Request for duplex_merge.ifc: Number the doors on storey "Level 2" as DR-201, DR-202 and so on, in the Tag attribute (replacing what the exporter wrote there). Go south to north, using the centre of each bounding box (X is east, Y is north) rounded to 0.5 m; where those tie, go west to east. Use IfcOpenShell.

First a look at what the model holds.

```python
import ifcopenshell
import ifcopenshell.util.element
import ifcopenshell.util.placement

model = ifcopenshell.open("duplex_merge.ifc")
print(model.schema)
storey = next(s for s in model.by_type("IfcBuildingStorey") if s.Name == "Level 2")
doors = [e for e in ifcopenshell.util.element.get_decomposition(storey) if e.is_a("IfcDoor")]
for e in sorted(doors, key=lambda e: e.id()):
    origin = ifcopenshell.util.placement.get_local_placement(e.ObjectPlacement)[:3, 3]
    print(e.id(), e.Tag, e.Name, origin.round(2) + 0.0, sep=" | ")
```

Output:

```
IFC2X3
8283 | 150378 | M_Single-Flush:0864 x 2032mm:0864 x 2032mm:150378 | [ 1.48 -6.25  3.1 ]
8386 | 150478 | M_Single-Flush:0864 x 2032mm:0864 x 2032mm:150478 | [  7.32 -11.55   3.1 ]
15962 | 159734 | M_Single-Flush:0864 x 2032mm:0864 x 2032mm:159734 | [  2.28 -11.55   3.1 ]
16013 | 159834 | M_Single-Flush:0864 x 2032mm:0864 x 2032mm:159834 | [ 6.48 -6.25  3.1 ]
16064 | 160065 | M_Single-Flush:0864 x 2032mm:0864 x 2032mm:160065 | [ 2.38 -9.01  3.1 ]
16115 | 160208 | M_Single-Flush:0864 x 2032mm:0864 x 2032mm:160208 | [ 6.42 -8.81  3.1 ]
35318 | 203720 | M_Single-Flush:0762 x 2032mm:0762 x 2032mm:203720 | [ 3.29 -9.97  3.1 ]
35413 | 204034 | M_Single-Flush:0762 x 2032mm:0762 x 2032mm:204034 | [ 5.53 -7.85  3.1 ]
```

```python
import ifcopenshell
import ifcopenshell.geom
import ifcopenshell.util.element
import ifcopenshell.util.shape

model = ifcopenshell.open("duplex_merge.ifc")
settings = ifcopenshell.geom.settings()
settings.set("use-world-coords", True)


def centre(element):
    shape = ifcopenshell.geom.create_shape(settings, element)
    return ifcopenshell.util.shape.get_bbox_centroid(shape.geometry)


storey = next(s for s in model.by_type("IfcBuildingStorey") if s.Name == "Level 2")
doors = [e for e in ifcopenshell.util.element.get_decomposition(storey) if e.is_a("IfcDoor")]

# Insertion points can sit at a corner or the storey origin, so sort by the geometry (in metres).
centres = {e: centre(e) for e in doors}
doors.sort(key=lambda e: (round(centres[e][1] / 0.5), centres[e][0]))

for i, e in enumerate(doors, start=1):
    number = f"DR-2{i:02d}"
    e.Tag = number
    print(e.id(), number)

model.write("duplex_merge-out.ifc")
```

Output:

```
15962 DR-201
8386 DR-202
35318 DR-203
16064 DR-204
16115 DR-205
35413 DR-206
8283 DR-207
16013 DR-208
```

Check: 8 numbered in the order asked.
